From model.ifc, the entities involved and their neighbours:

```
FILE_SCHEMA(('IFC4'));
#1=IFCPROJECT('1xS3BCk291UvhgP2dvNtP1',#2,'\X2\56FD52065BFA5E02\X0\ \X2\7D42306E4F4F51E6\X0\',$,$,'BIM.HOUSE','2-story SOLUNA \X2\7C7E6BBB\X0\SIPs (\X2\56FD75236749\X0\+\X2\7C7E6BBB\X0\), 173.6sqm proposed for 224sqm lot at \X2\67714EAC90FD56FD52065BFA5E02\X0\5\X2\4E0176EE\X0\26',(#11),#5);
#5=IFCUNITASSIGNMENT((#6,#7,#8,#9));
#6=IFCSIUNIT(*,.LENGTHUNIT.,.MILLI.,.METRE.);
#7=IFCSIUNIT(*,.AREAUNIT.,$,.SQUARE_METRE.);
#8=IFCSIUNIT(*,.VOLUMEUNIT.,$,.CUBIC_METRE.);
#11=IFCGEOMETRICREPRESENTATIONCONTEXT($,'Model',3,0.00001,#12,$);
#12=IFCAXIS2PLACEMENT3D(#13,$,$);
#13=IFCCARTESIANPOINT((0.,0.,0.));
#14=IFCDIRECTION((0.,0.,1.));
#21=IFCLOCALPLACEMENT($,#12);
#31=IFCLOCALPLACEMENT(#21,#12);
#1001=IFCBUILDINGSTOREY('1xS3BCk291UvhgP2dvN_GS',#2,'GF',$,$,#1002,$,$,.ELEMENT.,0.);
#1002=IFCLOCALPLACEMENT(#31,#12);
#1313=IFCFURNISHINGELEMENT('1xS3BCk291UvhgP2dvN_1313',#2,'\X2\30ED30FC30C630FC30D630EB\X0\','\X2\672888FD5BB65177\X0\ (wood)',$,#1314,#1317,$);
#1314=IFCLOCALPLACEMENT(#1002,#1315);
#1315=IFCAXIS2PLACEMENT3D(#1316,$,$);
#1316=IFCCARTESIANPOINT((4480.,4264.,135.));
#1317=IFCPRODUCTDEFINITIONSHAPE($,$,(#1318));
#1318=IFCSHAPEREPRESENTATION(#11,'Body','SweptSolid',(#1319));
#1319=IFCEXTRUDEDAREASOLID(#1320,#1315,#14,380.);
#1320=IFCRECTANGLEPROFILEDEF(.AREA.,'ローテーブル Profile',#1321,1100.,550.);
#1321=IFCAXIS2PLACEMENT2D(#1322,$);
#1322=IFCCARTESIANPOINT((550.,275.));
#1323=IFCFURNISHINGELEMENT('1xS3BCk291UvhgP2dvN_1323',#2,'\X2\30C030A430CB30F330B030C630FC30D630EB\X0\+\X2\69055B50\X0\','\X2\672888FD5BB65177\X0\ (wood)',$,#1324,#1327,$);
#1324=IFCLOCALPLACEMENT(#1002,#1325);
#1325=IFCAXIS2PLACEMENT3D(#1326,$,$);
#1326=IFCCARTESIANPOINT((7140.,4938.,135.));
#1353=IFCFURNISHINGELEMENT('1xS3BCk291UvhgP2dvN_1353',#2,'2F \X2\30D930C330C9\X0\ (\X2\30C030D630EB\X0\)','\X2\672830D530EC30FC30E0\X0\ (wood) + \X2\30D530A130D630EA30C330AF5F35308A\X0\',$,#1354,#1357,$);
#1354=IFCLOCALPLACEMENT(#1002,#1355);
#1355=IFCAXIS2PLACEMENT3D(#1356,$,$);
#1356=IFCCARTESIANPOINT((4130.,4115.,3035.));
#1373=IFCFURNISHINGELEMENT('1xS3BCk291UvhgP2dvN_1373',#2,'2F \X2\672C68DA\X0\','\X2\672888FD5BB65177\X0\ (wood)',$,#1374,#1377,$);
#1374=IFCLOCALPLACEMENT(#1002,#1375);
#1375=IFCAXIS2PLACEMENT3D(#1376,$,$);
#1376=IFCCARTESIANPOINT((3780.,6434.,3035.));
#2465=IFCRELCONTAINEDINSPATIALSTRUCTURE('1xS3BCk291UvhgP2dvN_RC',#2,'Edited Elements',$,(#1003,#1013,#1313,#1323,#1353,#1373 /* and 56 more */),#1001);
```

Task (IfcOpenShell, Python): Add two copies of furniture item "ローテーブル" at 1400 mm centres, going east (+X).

```python
import numpy as np
import ifcopenshell
import ifcopenshell.api.geometry
import ifcopenshell.api.root
import ifcopenshell.util.element
import ifcopenshell.util.placement
import ifcopenshell.util.unit

model = ifcopenshell.open("model.ifc")
unit_scale = ifcopenshell.util.unit.calculate_unit_scale(model)


def reuse_history(source, copy):
    """copy_class also copies each property set's owner history, people and application; keep the originals."""
    for rel in copy.IsDefinedBy:
        if rel.is_a("IfcRelDefinesByProperties") and (history := rel.RelatingPropertyDefinition.OwnerHistory):
            rel.RelatingPropertyDefinition.OwnerHistory = source.OwnerHistory
            ifcopenshell.util.element.remove_deep2(model, history)


source = model.by_id(1313)
base = ifcopenshell.util.placement.get_local_placement(source.ObjectPlacement)
step = np.array([1.0, 0.0, 0.0]) * 1.4 / unit_scale

for i in range(1, 3):
    copy = ifcopenshell.api.root.copy_class(model, product=source)
    copy.Representation = ifcopenshell.util.element.copy_deep(
        model, source.Representation, exclude=["IfcGeometricRepresentationContext", "IfcRepresentationMap"]
    )
    reuse_history(source, copy)
    matrix = base.copy()
    matrix[:3, 3] += i * step
    print("added at", matrix[:3, 3].round(3) + 0.0)
    ifcopenshell.api.geometry.edit_object_placement(model, product=copy, matrix=matrix, is_si=False)

model.write("model_updated.ifc")
```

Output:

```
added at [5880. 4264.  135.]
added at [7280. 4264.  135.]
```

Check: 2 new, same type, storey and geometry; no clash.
